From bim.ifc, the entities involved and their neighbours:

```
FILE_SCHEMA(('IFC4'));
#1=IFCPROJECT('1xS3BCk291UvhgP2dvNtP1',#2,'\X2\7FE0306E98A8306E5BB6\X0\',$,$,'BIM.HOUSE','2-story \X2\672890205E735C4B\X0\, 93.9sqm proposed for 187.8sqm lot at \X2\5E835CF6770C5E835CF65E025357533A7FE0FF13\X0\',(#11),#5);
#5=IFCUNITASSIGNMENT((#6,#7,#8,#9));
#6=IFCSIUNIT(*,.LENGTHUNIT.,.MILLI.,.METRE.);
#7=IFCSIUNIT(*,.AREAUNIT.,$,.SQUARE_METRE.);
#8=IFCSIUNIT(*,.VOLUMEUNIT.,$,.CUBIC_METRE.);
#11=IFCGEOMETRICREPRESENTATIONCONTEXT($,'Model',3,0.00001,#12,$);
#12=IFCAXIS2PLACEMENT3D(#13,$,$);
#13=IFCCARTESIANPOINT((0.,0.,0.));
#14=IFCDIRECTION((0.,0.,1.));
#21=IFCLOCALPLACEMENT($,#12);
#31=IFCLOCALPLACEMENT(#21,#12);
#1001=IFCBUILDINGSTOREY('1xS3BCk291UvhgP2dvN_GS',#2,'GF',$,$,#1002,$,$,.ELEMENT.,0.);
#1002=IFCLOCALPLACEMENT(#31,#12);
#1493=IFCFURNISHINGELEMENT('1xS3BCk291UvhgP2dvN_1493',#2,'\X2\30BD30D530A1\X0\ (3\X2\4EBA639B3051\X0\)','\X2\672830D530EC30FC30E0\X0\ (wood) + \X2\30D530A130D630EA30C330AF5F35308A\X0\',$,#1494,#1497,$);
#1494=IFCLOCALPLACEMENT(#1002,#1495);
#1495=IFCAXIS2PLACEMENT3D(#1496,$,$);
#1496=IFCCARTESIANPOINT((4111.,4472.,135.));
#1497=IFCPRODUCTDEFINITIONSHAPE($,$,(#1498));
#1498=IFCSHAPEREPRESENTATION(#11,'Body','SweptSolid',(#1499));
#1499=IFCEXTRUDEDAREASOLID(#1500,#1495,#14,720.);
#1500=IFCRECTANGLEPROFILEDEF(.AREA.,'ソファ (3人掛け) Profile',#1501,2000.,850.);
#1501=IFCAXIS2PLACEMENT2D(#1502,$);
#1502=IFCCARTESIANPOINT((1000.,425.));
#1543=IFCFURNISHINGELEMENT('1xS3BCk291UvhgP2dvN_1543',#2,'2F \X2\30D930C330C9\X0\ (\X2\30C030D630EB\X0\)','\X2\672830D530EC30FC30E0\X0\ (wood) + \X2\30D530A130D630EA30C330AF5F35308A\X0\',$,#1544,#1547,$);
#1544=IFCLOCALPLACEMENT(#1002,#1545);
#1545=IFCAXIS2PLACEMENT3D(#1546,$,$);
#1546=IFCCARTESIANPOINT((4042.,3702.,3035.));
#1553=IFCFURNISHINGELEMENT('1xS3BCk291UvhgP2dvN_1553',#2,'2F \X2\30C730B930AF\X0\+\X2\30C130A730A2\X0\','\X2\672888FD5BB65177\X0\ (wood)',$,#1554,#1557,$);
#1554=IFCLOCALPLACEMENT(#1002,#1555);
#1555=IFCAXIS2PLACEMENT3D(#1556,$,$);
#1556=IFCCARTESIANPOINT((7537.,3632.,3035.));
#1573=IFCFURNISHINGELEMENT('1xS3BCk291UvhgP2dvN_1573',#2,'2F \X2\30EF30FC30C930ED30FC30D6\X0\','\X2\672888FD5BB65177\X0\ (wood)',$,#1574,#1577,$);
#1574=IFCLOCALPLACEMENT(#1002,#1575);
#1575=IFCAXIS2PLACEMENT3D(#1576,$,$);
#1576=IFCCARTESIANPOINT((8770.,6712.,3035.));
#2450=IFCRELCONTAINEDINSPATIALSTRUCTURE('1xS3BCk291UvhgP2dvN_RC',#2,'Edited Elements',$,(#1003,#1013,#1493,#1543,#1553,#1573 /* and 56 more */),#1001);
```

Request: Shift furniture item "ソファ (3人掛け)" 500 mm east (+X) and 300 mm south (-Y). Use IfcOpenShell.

```python
import ifcopenshell
import ifcopenshell.api.geometry
import ifcopenshell.util.placement
import ifcopenshell.util.unit

model = ifcopenshell.open("bim.ifc")
unit_scale = ifcopenshell.util.unit.calculate_unit_scale(model)

item = model.by_id(1493)
matrix = ifcopenshell.util.placement.get_local_placement(item.ObjectPlacement)
matrix[0, 3] += 0.5 / unit_scale
matrix[1, 3] -= 0.3 / unit_scale
ifcopenshell.api.geometry.edit_object_placement(model, product=item, matrix=matrix, is_si=False)

print(ifcopenshell.util.placement.get_local_placement(item.ObjectPlacement).round(3) + 0.0)

model.write("bim_v2.ifc")
```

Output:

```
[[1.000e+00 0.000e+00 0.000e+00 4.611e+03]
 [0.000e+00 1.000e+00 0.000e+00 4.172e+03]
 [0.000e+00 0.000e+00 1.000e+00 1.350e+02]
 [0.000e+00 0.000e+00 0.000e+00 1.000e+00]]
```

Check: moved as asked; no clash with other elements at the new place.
